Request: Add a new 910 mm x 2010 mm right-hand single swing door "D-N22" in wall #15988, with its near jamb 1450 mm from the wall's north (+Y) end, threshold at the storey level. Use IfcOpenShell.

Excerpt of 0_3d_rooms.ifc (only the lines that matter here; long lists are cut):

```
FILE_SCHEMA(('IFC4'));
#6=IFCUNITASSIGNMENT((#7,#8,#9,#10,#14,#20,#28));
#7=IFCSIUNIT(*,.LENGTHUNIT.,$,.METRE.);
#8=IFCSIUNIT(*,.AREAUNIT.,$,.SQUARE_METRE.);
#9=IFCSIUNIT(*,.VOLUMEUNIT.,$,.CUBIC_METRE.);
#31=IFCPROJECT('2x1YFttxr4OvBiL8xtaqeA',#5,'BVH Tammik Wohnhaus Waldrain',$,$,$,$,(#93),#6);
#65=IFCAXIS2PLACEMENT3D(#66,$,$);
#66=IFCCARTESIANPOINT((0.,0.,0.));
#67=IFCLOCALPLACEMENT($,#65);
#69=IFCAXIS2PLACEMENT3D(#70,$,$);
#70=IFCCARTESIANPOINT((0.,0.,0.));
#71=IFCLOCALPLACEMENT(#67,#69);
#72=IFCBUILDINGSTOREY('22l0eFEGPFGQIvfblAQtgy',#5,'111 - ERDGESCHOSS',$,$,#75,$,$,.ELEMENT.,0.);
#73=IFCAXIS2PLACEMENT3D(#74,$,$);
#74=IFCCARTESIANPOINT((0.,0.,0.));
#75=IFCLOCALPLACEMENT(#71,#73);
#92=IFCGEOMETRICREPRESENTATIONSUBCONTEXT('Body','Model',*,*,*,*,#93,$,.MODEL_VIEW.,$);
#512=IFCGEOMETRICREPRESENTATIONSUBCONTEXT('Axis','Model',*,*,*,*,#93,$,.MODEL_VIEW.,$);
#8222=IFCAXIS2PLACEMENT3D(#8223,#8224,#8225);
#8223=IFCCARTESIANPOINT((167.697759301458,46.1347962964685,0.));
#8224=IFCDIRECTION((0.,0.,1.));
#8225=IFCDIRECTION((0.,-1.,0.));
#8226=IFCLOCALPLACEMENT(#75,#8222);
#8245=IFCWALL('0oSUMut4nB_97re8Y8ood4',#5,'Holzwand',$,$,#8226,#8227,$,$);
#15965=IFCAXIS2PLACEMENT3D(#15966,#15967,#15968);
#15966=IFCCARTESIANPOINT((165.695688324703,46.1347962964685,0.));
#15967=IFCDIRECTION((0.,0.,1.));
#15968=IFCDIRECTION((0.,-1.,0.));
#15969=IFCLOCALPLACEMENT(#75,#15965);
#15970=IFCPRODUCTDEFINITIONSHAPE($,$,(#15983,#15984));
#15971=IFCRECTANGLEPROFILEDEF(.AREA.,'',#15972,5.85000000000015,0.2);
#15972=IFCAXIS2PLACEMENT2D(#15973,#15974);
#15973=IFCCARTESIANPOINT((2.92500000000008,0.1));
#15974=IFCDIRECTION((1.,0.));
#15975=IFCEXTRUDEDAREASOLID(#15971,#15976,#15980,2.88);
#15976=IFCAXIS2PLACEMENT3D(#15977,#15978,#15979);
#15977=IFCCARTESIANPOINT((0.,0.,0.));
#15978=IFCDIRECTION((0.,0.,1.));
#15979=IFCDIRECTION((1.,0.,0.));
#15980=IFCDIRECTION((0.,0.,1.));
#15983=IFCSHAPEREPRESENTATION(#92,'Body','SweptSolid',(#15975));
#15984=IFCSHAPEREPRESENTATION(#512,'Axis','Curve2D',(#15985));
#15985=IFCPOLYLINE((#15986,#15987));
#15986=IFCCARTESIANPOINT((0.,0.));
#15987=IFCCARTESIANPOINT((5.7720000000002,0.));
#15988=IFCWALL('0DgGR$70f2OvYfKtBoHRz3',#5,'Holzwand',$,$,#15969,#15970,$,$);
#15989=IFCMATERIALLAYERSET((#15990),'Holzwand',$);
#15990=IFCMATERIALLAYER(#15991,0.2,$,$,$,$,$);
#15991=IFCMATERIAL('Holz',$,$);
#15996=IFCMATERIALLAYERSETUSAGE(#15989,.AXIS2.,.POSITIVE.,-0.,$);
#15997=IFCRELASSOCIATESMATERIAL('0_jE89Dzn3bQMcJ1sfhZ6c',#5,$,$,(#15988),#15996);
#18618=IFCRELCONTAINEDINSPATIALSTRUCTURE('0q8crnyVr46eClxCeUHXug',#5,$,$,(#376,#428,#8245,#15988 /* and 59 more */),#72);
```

```python
import numpy as np
import ifcopenshell
import ifcopenshell.api.feature
import ifcopenshell.api.geometry
import ifcopenshell.api.root
import ifcopenshell.api.spatial
import ifcopenshell.geom
import ifcopenshell.util.element
import ifcopenshell.util.placement
import ifcopenshell.util.representation
import ifcopenshell.util.shape
import ifcopenshell.util.unit

model = ifcopenshell.open("0_3d_rooms.ifc")
unit_scale = ifcopenshell.util.unit.calculate_unit_scale(model)
settings = ifcopenshell.geom.settings()


def volume(element):
    """Net volume in cubic metres, openings subtracted."""
    shape = ifcopenshell.geom.create_shape(settings, element)
    return ifcopenshell.util.shape.get_volume(shape.geometry)


wall = model.by_guid("0DgGR$70f2OvYfKtBoHRz3")
storey = ifcopenshell.util.element.get_container(wall, ifc_class="IfcBuildingStorey")
context = ifcopenshell.util.representation.get_context(model, "Model", "Body", "MODEL_VIEW")
before = volume(wall)

width, height, from_end, sill = 0.91, 2.01, 1.45, 0.0  # metres

# The wall runs along its own X axis, and the end named is its -X end.
wall_shape = ifcopenshell.geom.create_shape(settings, wall)
x, y, z = ifcopenshell.util.shape.get_vertices(wall_shape.geometry).T
start = x.min() + from_end
face, thickness = float(y.min()), float(y.max() - y.min())
wall_matrix = ifcopenshell.util.placement.get_local_placement(wall.ObjectPlacement)
level = ifcopenshell.util.placement.get_local_placement(storey.ObjectPlacement)[2, 3]


def in_wall(x, y):
    """Placement at x, y metres in the wall's axes, at sill height."""
    matrix = wall_matrix.copy()
    matrix[:, 3] = wall_matrix @ np.array([x / unit_scale, y / unit_scale, 0.0, 1.0])
    matrix[2, 3] = level + sill / unit_scale
    return matrix


# Opening: a box that overshoots both wall faces by 50 mm.
opening = ifcopenshell.api.root.create_entity(model, ifc_class="IfcOpeningElement", predefined_type="OPENING")
box = ifcopenshell.api.geometry.add_wall_representation(
    model, context=context, length=width, height=height, thickness=thickness + 0.1
)
ifcopenshell.api.geometry.assign_representation(model, product=opening, representation=box)
ifcopenshell.api.geometry.edit_object_placement(model, product=opening, matrix=in_wall(start, face - 0.05), is_si=False)
ifcopenshell.api.feature.add_feature(model, feature=opening, element=wall)

door = ifcopenshell.api.root.create_entity(model, ifc_class="IfcDoor", name="D-N22", predefined_type="DOOR")
door.OverallWidth, door.OverallHeight = width / unit_scale, height / unit_scale
door.OperationType = "SINGLE_SWING_RIGHT"
body = ifcopenshell.api.geometry.add_door_representation(
    model,
    context=context,
    overall_width=door.OverallWidth,
    overall_height=door.OverallHeight,
    operation_type="SINGLE_SWING_RIGHT",
    lining_properties={"LiningDepth": thickness / unit_scale, "ThresholdDepth": thickness / unit_scale},
)
ifcopenshell.api.geometry.assign_representation(model, product=door, representation=body)
ifcopenshell.api.spatial.assign_container(model, products=[door], relating_structure=storey)
ifcopenshell.api.feature.add_filling(model, opening=opening, element=door)

# The lining spans the wall, so the door starts at the wall face.
ifcopenshell.api.geometry.edit_object_placement(model, product=door, matrix=in_wall(start, face), is_si=False)

after = volume(wall)

print(f"wall volume {before:.3f} -> {after:.3f} m3")

model.write("0_3d_rooms_rev.ifc")
```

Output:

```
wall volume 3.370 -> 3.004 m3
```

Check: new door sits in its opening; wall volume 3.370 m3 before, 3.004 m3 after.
